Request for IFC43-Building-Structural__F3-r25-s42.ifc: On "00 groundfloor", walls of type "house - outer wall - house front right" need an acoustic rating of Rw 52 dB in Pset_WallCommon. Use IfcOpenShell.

First a look at what the model holds.

```python
import ifcopenshell
import ifcopenshell.util.element

model = ifcopenshell.open("IFC43-Building-Structural__F3-r25-s42.ifc")
print(model.schema)
storey = next(s for s in model.by_type("IfcBuildingStorey") if s.Name == "00 groundfloor")
walls = [e for e in ifcopenshell.util.element.get_decomposition(storey) if e.is_a("IfcWall")]
seen = {}
for e in walls:
    element_type = ifcopenshell.util.element.get_type(e)
    key = (element_type.Name if element_type != e and element_type else None, ifcopenshell.util.element.get_pset(e, "Pset_WallCommon", "AcousticRating"))
    seen[key] = seen.get(key, 0) + 1
for (name, value), count in sorted(seen.items(), key=str):
    print(count, "x", name, "|", value)
```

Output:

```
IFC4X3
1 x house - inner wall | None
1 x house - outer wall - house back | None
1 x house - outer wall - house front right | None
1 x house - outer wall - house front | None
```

```python
import ifcopenshell
import ifcopenshell.api.pset
import ifcopenshell.util.element

model = ifcopenshell.open("IFC43-Building-Structural__F3-r25-s42.ifc")

storey = next(s for s in model.by_type("IfcBuildingStorey") if s.Name == "00 groundfloor")
walls = [e for e in ifcopenshell.util.element.get_decomposition(storey) if e.is_a("IfcWall")]

count = 0
for e in walls:
    element_type = ifcopenshell.util.element.get_type(e)
    if element_type in (None, e) or element_type.Name != "house - outer wall - house front right":
        continue
    # add_pset returns the element's existing set when there is one.
    pset = ifcopenshell.api.pset.add_pset(model, product=e, name="Pset_WallCommon")
    ifcopenshell.api.pset.edit_pset(model, pset=pset, properties={"AcousticRating": "Rw 52 dB"})
    count += 1

print(count, "walls updated")

model.write("IFC43-Building-Structural__F3-r25-s42_edited.ifc")
```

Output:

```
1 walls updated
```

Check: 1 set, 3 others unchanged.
